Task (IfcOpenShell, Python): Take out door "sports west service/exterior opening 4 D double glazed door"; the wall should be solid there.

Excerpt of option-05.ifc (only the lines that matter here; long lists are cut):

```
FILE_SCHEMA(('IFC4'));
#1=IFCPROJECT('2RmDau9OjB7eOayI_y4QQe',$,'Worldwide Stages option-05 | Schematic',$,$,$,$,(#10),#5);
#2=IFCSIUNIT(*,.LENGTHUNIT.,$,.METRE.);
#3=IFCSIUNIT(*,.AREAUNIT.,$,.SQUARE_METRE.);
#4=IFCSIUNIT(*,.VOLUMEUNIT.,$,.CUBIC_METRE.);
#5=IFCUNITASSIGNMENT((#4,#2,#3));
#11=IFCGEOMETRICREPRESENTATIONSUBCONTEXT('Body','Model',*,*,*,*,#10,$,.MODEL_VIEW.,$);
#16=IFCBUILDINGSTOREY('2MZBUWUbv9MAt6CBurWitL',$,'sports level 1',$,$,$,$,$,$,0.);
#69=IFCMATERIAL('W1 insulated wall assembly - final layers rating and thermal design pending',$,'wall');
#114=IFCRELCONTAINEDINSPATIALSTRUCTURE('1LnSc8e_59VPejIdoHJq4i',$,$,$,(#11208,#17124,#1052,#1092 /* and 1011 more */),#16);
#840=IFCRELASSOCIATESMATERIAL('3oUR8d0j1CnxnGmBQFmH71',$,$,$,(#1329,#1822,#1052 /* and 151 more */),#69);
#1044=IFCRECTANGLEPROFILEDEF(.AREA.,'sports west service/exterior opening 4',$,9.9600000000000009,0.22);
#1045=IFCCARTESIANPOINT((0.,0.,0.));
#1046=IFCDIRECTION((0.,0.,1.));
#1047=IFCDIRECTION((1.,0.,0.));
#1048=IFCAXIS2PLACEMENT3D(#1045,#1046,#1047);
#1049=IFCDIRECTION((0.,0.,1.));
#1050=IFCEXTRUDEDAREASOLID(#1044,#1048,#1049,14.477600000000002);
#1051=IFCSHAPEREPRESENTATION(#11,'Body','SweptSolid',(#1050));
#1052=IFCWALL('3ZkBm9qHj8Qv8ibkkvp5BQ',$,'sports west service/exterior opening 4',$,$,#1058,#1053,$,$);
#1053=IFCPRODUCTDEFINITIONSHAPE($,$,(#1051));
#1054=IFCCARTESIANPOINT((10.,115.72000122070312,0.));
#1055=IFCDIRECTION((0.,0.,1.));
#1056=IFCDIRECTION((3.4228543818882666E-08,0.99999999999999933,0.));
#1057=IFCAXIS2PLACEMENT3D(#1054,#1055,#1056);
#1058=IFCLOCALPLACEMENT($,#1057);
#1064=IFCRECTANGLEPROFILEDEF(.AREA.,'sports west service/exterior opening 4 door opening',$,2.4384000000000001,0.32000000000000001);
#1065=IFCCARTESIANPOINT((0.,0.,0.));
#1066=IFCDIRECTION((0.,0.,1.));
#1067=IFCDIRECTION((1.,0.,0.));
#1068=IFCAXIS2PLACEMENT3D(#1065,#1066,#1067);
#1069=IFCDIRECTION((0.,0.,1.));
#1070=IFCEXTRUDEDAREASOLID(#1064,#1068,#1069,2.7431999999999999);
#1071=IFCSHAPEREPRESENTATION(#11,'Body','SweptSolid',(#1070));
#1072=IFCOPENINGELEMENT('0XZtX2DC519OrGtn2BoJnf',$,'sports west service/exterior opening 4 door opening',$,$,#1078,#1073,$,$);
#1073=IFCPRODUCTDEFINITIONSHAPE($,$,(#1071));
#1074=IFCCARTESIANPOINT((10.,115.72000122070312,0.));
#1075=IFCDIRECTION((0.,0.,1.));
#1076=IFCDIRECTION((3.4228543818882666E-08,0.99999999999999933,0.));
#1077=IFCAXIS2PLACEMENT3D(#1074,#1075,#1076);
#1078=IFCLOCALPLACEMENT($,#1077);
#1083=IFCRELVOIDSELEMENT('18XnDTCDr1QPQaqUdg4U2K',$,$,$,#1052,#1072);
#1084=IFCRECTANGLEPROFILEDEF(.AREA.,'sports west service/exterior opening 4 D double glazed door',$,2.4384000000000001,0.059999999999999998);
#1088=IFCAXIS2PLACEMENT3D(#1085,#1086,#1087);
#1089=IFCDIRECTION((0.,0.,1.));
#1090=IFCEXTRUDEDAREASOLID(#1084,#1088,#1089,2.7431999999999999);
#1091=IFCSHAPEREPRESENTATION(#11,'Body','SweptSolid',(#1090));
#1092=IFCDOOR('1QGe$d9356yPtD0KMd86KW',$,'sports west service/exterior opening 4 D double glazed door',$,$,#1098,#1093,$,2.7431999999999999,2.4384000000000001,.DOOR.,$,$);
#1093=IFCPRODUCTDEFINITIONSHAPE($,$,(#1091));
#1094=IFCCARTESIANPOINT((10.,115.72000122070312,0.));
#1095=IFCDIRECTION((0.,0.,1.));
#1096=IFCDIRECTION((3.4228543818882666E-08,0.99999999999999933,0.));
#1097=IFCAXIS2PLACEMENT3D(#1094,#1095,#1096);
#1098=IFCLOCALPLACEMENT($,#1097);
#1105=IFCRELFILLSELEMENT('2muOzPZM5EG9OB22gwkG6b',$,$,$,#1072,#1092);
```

```python
import ifcopenshell
import ifcopenshell.api.feature
import ifcopenshell.api.root
import ifcopenshell.geom
import ifcopenshell.util.shape

model = ifcopenshell.open("option-05.ifc")
settings = ifcopenshell.geom.settings()


def volume(element):
    """Net volume in cubic metres, openings subtracted."""
    shape = ifcopenshell.geom.create_shape(settings, element)
    return ifcopenshell.util.shape.get_volume(shape.geometry)


door = model.by_guid("1QGe$d9356yPtD0KMd86KW")
opening = door.FillsVoids[0].RelatingOpeningElement
wall = opening.VoidsElements[0].RelatingBuildingElement
before = volume(wall)

ifcopenshell.api.root.remove_product(model, product=door)
ifcopenshell.api.feature.remove_feature(model, feature=opening)

after = volume(wall)

print(f"wall volume {before:.3f} -> {after:.3f} m3")

model.write("option-05_edited.ifc")
```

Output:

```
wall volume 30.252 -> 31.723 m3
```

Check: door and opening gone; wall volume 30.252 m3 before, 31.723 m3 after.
